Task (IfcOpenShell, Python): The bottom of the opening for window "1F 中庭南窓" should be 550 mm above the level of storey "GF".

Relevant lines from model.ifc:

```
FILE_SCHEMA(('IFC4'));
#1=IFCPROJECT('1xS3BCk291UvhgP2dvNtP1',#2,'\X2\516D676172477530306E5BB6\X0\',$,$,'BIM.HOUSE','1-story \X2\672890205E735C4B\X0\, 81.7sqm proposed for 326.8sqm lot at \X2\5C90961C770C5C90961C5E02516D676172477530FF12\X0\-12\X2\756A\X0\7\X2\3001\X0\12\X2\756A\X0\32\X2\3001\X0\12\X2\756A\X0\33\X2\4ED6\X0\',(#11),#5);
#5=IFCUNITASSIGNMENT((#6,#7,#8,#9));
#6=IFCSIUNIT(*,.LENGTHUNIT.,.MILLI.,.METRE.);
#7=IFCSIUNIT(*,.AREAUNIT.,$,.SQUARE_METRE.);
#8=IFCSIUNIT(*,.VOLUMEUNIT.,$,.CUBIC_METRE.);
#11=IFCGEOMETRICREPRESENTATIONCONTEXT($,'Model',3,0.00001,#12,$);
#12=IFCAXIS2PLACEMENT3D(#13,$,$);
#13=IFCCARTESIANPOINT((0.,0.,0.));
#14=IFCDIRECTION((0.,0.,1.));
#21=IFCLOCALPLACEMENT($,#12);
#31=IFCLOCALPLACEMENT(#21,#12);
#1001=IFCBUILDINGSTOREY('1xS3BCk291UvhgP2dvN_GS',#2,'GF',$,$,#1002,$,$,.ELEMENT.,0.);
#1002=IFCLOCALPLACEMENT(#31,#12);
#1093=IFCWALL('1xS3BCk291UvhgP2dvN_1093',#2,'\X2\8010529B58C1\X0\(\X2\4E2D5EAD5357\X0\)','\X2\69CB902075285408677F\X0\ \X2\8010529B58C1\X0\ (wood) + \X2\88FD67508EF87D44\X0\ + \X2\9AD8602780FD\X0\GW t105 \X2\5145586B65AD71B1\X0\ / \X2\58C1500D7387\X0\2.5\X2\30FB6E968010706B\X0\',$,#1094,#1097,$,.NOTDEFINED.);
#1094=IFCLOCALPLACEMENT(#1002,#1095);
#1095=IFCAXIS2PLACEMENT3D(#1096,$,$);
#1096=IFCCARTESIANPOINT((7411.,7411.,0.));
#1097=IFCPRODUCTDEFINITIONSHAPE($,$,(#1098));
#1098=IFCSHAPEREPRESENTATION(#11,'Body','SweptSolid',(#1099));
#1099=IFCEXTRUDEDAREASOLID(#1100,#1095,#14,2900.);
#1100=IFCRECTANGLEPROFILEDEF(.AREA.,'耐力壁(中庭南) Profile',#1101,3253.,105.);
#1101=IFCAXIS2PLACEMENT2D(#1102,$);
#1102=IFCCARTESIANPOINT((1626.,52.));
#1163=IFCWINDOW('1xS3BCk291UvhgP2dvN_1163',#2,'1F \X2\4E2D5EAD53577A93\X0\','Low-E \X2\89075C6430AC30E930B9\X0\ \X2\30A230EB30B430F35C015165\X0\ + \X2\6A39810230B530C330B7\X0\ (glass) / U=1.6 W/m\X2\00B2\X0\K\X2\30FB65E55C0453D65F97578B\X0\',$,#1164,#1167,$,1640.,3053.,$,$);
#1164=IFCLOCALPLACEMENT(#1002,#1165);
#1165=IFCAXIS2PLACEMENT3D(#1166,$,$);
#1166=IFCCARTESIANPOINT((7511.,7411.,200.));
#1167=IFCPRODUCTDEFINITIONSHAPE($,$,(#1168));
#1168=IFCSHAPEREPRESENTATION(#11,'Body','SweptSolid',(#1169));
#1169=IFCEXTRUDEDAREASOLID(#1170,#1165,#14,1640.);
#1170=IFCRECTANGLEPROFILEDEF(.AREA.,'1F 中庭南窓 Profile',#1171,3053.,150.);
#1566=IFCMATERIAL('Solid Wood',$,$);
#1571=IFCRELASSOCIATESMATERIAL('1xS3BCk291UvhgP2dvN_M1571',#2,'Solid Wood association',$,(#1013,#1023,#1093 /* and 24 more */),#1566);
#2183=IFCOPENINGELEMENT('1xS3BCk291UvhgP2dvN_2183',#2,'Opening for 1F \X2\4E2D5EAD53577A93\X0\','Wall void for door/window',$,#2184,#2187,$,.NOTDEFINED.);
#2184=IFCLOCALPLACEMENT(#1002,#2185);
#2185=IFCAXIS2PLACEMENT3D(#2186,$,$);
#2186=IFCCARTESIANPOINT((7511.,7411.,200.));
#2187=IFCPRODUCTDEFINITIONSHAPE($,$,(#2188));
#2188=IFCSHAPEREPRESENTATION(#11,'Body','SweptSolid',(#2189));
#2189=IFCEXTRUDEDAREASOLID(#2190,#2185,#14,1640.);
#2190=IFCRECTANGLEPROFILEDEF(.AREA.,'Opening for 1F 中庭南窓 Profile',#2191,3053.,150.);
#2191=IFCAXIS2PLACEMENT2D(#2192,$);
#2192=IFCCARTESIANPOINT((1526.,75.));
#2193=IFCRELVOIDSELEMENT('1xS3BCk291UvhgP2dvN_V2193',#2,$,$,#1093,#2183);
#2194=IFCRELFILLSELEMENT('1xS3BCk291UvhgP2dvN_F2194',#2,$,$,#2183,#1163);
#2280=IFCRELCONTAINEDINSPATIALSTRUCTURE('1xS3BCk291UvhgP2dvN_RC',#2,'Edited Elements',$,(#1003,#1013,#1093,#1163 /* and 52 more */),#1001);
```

```python
import numpy as np
import ifcopenshell
import ifcopenshell.api.geometry
import ifcopenshell.geom
import ifcopenshell.util.element
import ifcopenshell.util.placement
import ifcopenshell.util.shape
import ifcopenshell.util.unit

model = ifcopenshell.open("model.ifc")
unit_scale = ifcopenshell.util.unit.calculate_unit_scale(model)

window = model.by_guid("1xS3BCk291UvhgP2dvN_1163")
opening = window.FillsVoids[0].RelatingOpeningElement
storey = ifcopenshell.util.element.get_container(window, ifc_class="IfcBuildingStorey")
level = ifcopenshell.util.placement.get_local_placement(storey.ObjectPlacement)[2, 3]

# The opening's origin need not be at the sill, so measure its lowest point.
shape = ifcopenshell.geom.create_shape(ifcopenshell.geom.settings(), opening)
bottom = ifcopenshell.util.shape.get_shape_bottom_elevation(shape, shape.geometry) / unit_scale
dz = level + 0.55 / unit_scale - bottom

shift = np.array([0.0, 0.0, dz])
# The window is not placed relative to its opening, so move both.
for product in (opening, window):
    matrix = ifcopenshell.util.placement.get_local_placement(product.ObjectPlacement)
    matrix[:3, 3] += shift
    ifcopenshell.api.geometry.edit_object_placement(model, product=product, matrix=matrix, is_si=False)

print(f"moved by {dz * unit_scale:+.3f} m")

model.write("model_updated.ifc")
```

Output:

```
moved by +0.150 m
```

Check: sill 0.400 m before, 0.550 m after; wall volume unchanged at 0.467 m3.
